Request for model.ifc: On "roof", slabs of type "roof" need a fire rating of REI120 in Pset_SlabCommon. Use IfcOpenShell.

First a look at what the model holds.

```python
import ifcopenshell
import ifcopenshell.util.element

model = ifcopenshell.open("model.ifc")
print(model.schema)
storey = next(s for s in model.by_type("IfcBuildingStorey") if s.Name == "roof")
slabs = [e for e in ifcopenshell.util.element.get_decomposition(storey) if e.is_a("IfcSlab")]
seen = {}
for e in slabs:
    element_type = ifcopenshell.util.element.get_type(e)
    key = (element_type.Name if element_type != e and element_type else None, ifcopenshell.util.element.get_pset(e, "Pset_SlabCommon", "FireRating"))
    seen[key] = seen.get(key, 0) + 1
for (name, value), count in sorted(seen.items(), key=str):
    print(count, "x", name, "|", value)
```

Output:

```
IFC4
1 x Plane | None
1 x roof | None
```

```python
import ifcopenshell
import ifcopenshell.api.pset
import ifcopenshell.util.element

model = ifcopenshell.open("model.ifc")

storey = next(s for s in model.by_type("IfcBuildingStorey") if s.Name == "roof")
slabs = [e for e in ifcopenshell.util.element.get_decomposition(storey) if e.is_a("IfcSlab")]

count = 0
for e in slabs:
    element_type = ifcopenshell.util.element.get_type(e)
    if element_type in (None, e) or element_type.Name != "roof":
        continue
    # add_pset returns the element's existing set when there is one.
    pset = ifcopenshell.api.pset.add_pset(model, product=e, name="Pset_SlabCommon")
    ifcopenshell.api.pset.edit_pset(model, pset=pset, properties={"FireRating": "REI120"})
    count += 1

print(count, "slabs updated")

model.write("model_v2.ifc")
```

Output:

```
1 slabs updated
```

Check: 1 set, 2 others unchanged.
